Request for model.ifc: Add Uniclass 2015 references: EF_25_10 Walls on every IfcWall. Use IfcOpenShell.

First a look at what the model holds.

```python
import ifcopenshell

model = ifcopenshell.open("model.ifc")
print(model.schema)
print("classifications:", [c.Name for c in model.by_type("IfcClassification")])
for ifc_class in ("IfcDoor", "IfcRoof", "IfcStair", "IfcWall", "IfcWindow"):
    print(ifc_class, len(model.by_type(ifc_class)))
```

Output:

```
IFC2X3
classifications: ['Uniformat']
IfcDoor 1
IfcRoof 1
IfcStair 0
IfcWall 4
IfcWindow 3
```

```python
import ifcopenshell
import ifcopenshell.api.classification

model = ifcopenshell.open("model.ifc")

# IFC2X3 requires Source and Edition and has no link from the project to the system.
system = model.create_entity("IfcClassification", Source="NBS", Edition="2015", Name="Uniclass 2015")

codes = {
    "IfcWall": ("EF_25_10", "Walls"),
}
for ifc_class, (code, name) in codes.items():
    products = model.by_type(ifc_class)
    ifcopenshell.api.classification.add_reference(
        model, products=products, classification=system, identification=code, name=name
    )
    print(code, len(products))

model.write("model_rev.ifc")
```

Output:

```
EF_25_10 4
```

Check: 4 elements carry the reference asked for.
